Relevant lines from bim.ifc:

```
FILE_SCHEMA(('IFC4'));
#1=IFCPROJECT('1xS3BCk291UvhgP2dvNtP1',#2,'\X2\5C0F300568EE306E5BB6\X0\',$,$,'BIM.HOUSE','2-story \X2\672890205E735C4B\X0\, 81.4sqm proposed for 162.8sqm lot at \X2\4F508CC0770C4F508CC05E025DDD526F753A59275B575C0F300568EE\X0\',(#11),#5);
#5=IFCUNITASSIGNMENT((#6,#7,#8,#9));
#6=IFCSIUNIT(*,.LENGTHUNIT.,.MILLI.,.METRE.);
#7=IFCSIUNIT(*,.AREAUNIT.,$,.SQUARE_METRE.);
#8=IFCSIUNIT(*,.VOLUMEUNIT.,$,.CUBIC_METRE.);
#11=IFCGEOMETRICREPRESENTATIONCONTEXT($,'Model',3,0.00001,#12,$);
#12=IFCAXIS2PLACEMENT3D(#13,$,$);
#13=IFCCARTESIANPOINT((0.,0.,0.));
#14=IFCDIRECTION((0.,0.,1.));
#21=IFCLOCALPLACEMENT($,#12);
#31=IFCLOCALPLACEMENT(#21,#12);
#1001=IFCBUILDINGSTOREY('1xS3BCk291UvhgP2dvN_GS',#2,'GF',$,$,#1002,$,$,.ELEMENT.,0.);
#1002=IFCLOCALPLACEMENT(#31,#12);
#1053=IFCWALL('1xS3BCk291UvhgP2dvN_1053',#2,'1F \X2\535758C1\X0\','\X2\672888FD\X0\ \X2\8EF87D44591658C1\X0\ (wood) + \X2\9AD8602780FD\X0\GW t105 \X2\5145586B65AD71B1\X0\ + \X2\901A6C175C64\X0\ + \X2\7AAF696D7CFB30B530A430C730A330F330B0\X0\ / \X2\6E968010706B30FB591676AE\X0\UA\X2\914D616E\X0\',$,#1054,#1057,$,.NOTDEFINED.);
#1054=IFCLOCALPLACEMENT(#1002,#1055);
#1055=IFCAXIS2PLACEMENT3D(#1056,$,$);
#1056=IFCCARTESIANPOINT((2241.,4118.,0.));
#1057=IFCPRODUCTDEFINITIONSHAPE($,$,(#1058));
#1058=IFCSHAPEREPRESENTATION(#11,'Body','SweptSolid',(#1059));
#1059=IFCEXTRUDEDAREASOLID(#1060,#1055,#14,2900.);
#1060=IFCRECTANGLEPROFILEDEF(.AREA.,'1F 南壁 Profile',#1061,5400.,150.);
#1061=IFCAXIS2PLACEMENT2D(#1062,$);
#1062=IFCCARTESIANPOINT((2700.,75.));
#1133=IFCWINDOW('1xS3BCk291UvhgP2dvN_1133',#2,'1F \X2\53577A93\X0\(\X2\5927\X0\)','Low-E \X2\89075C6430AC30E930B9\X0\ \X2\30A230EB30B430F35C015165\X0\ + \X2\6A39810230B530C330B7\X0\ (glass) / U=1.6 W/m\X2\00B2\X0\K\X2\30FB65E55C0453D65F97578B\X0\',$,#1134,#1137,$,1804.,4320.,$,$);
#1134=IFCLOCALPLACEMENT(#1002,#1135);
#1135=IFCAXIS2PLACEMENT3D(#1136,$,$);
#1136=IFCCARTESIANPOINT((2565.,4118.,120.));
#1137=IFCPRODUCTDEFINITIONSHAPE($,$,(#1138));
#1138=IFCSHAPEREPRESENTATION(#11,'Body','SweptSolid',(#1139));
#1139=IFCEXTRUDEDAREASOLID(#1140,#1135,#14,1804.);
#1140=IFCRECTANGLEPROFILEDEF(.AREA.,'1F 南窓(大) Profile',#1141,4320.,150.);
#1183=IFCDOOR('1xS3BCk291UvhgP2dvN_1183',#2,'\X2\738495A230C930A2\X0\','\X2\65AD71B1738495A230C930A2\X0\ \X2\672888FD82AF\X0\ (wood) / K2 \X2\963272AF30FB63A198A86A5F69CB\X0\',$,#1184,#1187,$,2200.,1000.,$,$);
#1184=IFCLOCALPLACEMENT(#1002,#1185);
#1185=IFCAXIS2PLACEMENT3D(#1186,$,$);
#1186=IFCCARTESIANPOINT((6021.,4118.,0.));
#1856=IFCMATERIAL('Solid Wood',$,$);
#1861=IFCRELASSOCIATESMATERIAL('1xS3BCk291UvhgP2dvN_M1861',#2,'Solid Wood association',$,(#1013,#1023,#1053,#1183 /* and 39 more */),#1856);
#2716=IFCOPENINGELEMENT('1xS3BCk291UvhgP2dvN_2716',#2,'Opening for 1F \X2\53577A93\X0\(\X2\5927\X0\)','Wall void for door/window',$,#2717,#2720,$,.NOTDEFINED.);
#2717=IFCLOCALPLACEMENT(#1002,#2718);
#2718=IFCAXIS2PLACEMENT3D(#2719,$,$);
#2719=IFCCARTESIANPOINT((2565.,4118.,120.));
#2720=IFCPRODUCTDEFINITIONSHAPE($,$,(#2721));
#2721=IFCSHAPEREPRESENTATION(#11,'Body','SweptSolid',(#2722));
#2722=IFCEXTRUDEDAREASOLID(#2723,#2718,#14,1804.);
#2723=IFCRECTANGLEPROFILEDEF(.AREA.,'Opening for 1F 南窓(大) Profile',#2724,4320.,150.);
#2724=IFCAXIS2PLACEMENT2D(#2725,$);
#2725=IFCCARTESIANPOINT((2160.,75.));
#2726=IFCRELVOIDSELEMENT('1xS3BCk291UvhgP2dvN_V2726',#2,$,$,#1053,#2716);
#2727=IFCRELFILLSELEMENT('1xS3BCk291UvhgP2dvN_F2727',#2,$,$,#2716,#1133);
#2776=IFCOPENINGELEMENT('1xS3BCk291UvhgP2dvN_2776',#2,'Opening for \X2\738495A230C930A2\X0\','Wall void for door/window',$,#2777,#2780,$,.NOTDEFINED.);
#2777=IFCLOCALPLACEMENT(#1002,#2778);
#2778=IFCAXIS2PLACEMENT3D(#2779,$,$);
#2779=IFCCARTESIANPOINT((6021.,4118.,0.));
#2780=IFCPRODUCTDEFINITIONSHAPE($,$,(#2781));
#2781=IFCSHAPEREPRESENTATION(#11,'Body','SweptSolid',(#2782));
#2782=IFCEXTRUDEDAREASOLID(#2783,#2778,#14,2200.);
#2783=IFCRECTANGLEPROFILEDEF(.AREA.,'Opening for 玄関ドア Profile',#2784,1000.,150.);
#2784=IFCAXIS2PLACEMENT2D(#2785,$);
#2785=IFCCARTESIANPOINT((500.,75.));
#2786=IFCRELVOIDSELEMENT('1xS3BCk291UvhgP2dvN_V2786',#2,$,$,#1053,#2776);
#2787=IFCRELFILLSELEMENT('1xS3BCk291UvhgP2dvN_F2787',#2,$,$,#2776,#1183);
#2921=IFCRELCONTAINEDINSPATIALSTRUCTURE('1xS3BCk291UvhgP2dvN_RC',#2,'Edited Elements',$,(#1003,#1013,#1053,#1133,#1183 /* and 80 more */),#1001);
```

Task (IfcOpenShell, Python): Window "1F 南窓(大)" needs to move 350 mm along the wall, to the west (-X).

```python
import ifcopenshell
import ifcopenshell.api.geometry
import ifcopenshell.util.placement

model = ifcopenshell.open("bim.ifc")

window = model.by_guid("1xS3BCk291UvhgP2dvN_1133")
opening = window.FillsVoids[0].RelatingOpeningElement
wall = opening.VoidsElements[0].RelatingBuildingElement

wall_matrix = ifcopenshell.util.placement.get_local_placement(wall.ObjectPlacement)
shift = wall_matrix[:3, 0] * -350.0
before = ifcopenshell.util.placement.get_local_placement(window.ObjectPlacement)[:3, 3].copy()

# The window is not placed relative to its opening, so move both.
for product in (opening, window):
    matrix = ifcopenshell.util.placement.get_local_placement(product.ObjectPlacement)
    matrix[:3, 3] += shift
    ifcopenshell.api.geometry.edit_object_placement(model, product=product, matrix=matrix, is_si=False)

after = ifcopenshell.util.placement.get_local_placement(window.ObjectPlacement)[:3, 3]
print("window moved by", (after - before).round(3) + 0.0)

model.write("bim_edited.ifc")
```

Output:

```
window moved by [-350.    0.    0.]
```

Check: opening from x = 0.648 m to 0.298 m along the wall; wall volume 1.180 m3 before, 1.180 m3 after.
